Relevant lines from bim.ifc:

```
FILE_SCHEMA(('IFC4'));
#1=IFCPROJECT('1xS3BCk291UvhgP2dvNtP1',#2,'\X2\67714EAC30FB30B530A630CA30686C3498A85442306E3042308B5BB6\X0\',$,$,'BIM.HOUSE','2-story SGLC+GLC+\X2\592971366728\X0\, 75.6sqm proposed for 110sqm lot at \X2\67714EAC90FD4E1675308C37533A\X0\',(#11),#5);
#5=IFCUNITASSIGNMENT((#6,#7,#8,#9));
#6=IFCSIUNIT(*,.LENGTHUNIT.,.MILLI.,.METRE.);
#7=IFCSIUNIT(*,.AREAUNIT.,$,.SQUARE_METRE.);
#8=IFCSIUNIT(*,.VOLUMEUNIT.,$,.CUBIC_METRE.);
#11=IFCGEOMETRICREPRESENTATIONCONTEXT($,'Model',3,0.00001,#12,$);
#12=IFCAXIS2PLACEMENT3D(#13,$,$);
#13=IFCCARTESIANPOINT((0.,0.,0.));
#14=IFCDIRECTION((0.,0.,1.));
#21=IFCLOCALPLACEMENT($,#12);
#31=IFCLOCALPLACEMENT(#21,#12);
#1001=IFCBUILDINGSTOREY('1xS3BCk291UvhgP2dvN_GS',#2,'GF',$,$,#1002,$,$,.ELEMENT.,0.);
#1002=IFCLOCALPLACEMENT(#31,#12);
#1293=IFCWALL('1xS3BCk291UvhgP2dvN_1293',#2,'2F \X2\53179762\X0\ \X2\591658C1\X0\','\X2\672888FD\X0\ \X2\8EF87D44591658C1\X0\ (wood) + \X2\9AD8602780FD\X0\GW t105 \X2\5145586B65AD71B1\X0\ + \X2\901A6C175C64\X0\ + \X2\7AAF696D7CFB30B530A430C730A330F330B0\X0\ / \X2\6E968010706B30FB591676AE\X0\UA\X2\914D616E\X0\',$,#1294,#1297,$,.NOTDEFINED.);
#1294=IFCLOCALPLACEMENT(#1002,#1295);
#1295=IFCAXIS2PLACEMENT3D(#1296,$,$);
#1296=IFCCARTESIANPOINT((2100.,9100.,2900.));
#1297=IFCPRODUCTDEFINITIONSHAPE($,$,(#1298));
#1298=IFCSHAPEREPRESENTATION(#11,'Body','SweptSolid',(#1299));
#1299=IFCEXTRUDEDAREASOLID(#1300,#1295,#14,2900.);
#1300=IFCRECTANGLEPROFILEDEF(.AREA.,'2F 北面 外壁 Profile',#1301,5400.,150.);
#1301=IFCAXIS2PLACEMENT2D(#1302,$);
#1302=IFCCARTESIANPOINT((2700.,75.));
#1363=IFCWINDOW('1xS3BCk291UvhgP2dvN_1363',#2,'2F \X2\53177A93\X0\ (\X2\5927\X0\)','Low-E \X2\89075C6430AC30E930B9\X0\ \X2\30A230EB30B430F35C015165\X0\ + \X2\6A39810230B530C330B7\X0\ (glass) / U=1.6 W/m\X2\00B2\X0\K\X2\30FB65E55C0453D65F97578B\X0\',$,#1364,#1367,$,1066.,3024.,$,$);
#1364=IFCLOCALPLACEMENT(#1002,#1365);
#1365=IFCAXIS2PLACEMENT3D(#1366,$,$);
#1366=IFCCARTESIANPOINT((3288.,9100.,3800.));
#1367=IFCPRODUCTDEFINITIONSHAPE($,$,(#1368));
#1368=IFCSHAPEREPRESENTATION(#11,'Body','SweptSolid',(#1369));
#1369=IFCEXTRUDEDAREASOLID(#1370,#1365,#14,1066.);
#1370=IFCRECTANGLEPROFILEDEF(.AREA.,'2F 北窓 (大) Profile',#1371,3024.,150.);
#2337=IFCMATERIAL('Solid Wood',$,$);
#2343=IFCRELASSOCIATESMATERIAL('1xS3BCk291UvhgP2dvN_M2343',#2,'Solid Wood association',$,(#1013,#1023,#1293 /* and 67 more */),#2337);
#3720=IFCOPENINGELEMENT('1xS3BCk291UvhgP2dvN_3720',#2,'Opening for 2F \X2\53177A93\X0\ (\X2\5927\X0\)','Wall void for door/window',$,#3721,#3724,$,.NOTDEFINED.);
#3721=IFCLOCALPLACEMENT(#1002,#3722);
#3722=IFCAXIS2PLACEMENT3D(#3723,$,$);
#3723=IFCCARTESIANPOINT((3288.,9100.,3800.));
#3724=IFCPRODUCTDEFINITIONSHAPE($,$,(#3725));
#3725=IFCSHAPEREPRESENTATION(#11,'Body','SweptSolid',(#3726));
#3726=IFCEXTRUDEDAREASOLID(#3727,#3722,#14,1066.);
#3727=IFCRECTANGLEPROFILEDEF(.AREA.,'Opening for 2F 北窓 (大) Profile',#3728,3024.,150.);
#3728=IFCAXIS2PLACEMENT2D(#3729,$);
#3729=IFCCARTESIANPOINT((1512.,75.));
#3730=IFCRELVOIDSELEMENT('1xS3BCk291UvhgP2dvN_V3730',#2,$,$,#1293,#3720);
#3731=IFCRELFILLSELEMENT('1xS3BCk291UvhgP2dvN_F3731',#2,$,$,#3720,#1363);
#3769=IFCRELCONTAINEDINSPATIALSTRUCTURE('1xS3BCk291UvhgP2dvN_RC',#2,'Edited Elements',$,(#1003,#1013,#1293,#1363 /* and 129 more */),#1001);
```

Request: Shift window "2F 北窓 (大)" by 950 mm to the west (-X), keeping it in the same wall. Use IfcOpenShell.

```python
import ifcopenshell
import ifcopenshell.api.geometry
import ifcopenshell.util.placement
import ifcopenshell.util.unit

model = ifcopenshell.open("bim.ifc")
unit_scale = ifcopenshell.util.unit.calculate_unit_scale(model)

window = model.by_guid("1xS3BCk291UvhgP2dvN_1363")
opening = window.FillsVoids[0].RelatingOpeningElement
wall = opening.VoidsElements[0].RelatingBuildingElement

wall_matrix = ifcopenshell.util.placement.get_local_placement(wall.ObjectPlacement)
shift = wall_matrix[:3, 0] * -0.95 / unit_scale
before = ifcopenshell.util.placement.get_local_placement(window.ObjectPlacement)[:3, 3].copy()

# The window is not placed relative to its opening, so move both.
for product in (opening, window):
    matrix = ifcopenshell.util.placement.get_local_placement(product.ObjectPlacement)
    matrix[:3, 3] += shift
    ifcopenshell.api.geometry.edit_object_placement(model, product=product, matrix=matrix, is_si=False)

after = ifcopenshell.util.placement.get_local_placement(window.ObjectPlacement)[:3, 3]
print("window moved by", (after - before).round(3) + 0.0)

model.write("bim_rev.ifc")
```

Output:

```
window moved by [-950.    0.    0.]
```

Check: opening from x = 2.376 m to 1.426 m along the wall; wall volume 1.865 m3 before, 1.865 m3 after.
